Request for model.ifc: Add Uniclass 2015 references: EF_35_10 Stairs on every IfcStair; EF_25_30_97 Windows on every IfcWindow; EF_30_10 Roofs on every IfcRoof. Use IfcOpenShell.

First a look at what the model holds.

```python
import ifcopenshell

model = ifcopenshell.open("model.ifc")
print(model.schema)
print("classifications:", [c.Name for c in model.by_type("IfcClassification")])
for ifc_class in ("IfcDoor", "IfcRoof", "IfcStair", "IfcWall", "IfcWindow"):
    print(ifc_class, len(model.by_type(ifc_class)))
```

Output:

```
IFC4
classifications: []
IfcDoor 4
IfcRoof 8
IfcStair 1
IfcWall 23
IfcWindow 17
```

```python
import ifcopenshell
import ifcopenshell.api.classification

model = ifcopenshell.open("model.ifc")

system = ifcopenshell.api.classification.add_classification(model, classification="Uniclass 2015")

codes = {
    "IfcStair": ("EF_35_10", "Stairs"),
    "IfcWindow": ("EF_25_30_97", "Windows"),
    "IfcRoof": ("EF_30_10", "Roofs"),
}
for ifc_class, (code, name) in codes.items():
    products = model.by_type(ifc_class)
    ifcopenshell.api.classification.add_reference(
        model, products=products, classification=system, identification=code, name=name
    )
    print(code, len(products))

model.write("model_v2.ifc")
```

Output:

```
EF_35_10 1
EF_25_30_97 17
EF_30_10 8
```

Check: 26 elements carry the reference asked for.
